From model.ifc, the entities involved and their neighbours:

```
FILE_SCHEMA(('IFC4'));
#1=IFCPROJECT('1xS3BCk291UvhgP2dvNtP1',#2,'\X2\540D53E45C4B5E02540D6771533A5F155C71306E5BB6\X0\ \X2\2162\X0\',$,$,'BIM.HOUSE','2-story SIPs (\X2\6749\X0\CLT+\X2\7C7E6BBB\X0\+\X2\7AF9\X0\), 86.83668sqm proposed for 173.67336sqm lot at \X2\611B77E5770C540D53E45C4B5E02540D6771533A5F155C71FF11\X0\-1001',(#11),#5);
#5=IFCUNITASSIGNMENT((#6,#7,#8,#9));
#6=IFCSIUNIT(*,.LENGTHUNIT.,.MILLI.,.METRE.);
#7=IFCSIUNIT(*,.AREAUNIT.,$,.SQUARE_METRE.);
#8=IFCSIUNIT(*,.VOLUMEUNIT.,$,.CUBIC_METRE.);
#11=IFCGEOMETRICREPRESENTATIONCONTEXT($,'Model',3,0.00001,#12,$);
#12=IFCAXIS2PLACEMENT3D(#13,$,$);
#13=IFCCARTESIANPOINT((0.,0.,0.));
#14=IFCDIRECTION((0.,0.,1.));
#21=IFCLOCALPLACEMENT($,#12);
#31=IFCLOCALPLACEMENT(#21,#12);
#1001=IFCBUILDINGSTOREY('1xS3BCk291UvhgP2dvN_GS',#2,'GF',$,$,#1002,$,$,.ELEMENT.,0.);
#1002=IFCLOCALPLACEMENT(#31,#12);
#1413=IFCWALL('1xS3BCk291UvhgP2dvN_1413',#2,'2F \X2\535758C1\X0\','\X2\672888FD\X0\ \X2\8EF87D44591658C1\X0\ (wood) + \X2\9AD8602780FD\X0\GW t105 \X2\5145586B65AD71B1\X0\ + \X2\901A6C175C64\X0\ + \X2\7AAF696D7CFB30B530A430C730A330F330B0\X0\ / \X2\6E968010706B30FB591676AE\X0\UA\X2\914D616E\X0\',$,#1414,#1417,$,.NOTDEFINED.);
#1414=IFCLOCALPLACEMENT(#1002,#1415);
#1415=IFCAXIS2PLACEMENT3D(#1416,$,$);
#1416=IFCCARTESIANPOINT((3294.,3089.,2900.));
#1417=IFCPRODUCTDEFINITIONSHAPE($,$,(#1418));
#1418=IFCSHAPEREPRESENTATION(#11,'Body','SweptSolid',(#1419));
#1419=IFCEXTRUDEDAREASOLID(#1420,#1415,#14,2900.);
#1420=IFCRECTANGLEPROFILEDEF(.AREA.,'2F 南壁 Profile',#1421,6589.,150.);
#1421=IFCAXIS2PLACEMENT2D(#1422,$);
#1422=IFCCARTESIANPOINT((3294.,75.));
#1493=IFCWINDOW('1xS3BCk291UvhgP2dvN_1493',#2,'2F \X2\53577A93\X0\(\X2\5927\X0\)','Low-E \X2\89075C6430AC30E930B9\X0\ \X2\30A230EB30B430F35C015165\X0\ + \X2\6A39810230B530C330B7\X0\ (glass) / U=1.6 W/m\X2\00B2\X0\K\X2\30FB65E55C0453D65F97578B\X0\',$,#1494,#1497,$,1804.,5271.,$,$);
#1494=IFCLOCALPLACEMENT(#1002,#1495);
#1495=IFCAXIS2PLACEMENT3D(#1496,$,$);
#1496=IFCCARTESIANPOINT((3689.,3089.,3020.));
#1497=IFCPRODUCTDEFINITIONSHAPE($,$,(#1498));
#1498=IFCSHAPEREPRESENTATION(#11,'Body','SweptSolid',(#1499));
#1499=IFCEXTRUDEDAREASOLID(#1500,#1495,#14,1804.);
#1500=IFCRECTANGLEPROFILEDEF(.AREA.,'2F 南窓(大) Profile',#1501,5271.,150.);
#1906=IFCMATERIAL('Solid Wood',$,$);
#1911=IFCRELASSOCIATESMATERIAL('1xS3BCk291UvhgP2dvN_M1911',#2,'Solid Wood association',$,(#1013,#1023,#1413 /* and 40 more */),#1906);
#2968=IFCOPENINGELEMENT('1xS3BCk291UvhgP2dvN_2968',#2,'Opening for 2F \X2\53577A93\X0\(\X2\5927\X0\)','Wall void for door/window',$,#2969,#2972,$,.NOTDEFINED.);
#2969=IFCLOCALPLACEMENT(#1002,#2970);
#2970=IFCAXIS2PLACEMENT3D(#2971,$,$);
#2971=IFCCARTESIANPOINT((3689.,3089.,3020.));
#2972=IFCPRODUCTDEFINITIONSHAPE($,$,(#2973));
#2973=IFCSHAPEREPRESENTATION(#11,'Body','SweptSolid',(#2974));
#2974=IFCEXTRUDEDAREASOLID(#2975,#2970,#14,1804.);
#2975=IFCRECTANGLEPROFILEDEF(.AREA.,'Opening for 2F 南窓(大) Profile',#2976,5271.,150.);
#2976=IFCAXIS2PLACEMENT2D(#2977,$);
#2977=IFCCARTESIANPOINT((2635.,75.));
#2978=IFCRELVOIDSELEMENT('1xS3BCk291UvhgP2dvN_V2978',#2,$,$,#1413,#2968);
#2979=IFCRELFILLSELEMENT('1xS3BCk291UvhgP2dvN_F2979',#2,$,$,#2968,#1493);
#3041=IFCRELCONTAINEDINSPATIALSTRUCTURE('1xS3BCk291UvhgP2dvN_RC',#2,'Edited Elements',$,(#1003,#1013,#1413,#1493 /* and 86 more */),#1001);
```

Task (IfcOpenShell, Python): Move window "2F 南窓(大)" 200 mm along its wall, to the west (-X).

```python
import ifcopenshell
import ifcopenshell.api.geometry
import ifcopenshell.util.placement
import ifcopenshell.util.unit

model = ifcopenshell.open("model.ifc")
unit_scale = ifcopenshell.util.unit.calculate_unit_scale(model)

window = model.by_id(1493)
opening = window.FillsVoids[0].RelatingOpeningElement
wall = opening.VoidsElements[0].RelatingBuildingElement

wall_matrix = ifcopenshell.util.placement.get_local_placement(wall.ObjectPlacement)
shift = wall_matrix[:3, 0] * -0.2 / unit_scale
before = ifcopenshell.util.placement.get_local_placement(window.ObjectPlacement)[:3, 3].copy()

# The window is not placed relative to its opening, so move both.
for product in (opening, window):
    matrix = ifcopenshell.util.placement.get_local_placement(product.ObjectPlacement)
    matrix[:3, 3] += shift
    ifcopenshell.api.geometry.edit_object_placement(model, product=product, matrix=matrix, is_si=False)

after = ifcopenshell.util.placement.get_local_placement(window.ObjectPlacement)[:3, 3]
print("window moved by", (after - before).round(3) + 0.0)

model.write("model_edited.ifc")
```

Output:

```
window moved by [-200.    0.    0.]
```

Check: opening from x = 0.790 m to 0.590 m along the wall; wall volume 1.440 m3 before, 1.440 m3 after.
